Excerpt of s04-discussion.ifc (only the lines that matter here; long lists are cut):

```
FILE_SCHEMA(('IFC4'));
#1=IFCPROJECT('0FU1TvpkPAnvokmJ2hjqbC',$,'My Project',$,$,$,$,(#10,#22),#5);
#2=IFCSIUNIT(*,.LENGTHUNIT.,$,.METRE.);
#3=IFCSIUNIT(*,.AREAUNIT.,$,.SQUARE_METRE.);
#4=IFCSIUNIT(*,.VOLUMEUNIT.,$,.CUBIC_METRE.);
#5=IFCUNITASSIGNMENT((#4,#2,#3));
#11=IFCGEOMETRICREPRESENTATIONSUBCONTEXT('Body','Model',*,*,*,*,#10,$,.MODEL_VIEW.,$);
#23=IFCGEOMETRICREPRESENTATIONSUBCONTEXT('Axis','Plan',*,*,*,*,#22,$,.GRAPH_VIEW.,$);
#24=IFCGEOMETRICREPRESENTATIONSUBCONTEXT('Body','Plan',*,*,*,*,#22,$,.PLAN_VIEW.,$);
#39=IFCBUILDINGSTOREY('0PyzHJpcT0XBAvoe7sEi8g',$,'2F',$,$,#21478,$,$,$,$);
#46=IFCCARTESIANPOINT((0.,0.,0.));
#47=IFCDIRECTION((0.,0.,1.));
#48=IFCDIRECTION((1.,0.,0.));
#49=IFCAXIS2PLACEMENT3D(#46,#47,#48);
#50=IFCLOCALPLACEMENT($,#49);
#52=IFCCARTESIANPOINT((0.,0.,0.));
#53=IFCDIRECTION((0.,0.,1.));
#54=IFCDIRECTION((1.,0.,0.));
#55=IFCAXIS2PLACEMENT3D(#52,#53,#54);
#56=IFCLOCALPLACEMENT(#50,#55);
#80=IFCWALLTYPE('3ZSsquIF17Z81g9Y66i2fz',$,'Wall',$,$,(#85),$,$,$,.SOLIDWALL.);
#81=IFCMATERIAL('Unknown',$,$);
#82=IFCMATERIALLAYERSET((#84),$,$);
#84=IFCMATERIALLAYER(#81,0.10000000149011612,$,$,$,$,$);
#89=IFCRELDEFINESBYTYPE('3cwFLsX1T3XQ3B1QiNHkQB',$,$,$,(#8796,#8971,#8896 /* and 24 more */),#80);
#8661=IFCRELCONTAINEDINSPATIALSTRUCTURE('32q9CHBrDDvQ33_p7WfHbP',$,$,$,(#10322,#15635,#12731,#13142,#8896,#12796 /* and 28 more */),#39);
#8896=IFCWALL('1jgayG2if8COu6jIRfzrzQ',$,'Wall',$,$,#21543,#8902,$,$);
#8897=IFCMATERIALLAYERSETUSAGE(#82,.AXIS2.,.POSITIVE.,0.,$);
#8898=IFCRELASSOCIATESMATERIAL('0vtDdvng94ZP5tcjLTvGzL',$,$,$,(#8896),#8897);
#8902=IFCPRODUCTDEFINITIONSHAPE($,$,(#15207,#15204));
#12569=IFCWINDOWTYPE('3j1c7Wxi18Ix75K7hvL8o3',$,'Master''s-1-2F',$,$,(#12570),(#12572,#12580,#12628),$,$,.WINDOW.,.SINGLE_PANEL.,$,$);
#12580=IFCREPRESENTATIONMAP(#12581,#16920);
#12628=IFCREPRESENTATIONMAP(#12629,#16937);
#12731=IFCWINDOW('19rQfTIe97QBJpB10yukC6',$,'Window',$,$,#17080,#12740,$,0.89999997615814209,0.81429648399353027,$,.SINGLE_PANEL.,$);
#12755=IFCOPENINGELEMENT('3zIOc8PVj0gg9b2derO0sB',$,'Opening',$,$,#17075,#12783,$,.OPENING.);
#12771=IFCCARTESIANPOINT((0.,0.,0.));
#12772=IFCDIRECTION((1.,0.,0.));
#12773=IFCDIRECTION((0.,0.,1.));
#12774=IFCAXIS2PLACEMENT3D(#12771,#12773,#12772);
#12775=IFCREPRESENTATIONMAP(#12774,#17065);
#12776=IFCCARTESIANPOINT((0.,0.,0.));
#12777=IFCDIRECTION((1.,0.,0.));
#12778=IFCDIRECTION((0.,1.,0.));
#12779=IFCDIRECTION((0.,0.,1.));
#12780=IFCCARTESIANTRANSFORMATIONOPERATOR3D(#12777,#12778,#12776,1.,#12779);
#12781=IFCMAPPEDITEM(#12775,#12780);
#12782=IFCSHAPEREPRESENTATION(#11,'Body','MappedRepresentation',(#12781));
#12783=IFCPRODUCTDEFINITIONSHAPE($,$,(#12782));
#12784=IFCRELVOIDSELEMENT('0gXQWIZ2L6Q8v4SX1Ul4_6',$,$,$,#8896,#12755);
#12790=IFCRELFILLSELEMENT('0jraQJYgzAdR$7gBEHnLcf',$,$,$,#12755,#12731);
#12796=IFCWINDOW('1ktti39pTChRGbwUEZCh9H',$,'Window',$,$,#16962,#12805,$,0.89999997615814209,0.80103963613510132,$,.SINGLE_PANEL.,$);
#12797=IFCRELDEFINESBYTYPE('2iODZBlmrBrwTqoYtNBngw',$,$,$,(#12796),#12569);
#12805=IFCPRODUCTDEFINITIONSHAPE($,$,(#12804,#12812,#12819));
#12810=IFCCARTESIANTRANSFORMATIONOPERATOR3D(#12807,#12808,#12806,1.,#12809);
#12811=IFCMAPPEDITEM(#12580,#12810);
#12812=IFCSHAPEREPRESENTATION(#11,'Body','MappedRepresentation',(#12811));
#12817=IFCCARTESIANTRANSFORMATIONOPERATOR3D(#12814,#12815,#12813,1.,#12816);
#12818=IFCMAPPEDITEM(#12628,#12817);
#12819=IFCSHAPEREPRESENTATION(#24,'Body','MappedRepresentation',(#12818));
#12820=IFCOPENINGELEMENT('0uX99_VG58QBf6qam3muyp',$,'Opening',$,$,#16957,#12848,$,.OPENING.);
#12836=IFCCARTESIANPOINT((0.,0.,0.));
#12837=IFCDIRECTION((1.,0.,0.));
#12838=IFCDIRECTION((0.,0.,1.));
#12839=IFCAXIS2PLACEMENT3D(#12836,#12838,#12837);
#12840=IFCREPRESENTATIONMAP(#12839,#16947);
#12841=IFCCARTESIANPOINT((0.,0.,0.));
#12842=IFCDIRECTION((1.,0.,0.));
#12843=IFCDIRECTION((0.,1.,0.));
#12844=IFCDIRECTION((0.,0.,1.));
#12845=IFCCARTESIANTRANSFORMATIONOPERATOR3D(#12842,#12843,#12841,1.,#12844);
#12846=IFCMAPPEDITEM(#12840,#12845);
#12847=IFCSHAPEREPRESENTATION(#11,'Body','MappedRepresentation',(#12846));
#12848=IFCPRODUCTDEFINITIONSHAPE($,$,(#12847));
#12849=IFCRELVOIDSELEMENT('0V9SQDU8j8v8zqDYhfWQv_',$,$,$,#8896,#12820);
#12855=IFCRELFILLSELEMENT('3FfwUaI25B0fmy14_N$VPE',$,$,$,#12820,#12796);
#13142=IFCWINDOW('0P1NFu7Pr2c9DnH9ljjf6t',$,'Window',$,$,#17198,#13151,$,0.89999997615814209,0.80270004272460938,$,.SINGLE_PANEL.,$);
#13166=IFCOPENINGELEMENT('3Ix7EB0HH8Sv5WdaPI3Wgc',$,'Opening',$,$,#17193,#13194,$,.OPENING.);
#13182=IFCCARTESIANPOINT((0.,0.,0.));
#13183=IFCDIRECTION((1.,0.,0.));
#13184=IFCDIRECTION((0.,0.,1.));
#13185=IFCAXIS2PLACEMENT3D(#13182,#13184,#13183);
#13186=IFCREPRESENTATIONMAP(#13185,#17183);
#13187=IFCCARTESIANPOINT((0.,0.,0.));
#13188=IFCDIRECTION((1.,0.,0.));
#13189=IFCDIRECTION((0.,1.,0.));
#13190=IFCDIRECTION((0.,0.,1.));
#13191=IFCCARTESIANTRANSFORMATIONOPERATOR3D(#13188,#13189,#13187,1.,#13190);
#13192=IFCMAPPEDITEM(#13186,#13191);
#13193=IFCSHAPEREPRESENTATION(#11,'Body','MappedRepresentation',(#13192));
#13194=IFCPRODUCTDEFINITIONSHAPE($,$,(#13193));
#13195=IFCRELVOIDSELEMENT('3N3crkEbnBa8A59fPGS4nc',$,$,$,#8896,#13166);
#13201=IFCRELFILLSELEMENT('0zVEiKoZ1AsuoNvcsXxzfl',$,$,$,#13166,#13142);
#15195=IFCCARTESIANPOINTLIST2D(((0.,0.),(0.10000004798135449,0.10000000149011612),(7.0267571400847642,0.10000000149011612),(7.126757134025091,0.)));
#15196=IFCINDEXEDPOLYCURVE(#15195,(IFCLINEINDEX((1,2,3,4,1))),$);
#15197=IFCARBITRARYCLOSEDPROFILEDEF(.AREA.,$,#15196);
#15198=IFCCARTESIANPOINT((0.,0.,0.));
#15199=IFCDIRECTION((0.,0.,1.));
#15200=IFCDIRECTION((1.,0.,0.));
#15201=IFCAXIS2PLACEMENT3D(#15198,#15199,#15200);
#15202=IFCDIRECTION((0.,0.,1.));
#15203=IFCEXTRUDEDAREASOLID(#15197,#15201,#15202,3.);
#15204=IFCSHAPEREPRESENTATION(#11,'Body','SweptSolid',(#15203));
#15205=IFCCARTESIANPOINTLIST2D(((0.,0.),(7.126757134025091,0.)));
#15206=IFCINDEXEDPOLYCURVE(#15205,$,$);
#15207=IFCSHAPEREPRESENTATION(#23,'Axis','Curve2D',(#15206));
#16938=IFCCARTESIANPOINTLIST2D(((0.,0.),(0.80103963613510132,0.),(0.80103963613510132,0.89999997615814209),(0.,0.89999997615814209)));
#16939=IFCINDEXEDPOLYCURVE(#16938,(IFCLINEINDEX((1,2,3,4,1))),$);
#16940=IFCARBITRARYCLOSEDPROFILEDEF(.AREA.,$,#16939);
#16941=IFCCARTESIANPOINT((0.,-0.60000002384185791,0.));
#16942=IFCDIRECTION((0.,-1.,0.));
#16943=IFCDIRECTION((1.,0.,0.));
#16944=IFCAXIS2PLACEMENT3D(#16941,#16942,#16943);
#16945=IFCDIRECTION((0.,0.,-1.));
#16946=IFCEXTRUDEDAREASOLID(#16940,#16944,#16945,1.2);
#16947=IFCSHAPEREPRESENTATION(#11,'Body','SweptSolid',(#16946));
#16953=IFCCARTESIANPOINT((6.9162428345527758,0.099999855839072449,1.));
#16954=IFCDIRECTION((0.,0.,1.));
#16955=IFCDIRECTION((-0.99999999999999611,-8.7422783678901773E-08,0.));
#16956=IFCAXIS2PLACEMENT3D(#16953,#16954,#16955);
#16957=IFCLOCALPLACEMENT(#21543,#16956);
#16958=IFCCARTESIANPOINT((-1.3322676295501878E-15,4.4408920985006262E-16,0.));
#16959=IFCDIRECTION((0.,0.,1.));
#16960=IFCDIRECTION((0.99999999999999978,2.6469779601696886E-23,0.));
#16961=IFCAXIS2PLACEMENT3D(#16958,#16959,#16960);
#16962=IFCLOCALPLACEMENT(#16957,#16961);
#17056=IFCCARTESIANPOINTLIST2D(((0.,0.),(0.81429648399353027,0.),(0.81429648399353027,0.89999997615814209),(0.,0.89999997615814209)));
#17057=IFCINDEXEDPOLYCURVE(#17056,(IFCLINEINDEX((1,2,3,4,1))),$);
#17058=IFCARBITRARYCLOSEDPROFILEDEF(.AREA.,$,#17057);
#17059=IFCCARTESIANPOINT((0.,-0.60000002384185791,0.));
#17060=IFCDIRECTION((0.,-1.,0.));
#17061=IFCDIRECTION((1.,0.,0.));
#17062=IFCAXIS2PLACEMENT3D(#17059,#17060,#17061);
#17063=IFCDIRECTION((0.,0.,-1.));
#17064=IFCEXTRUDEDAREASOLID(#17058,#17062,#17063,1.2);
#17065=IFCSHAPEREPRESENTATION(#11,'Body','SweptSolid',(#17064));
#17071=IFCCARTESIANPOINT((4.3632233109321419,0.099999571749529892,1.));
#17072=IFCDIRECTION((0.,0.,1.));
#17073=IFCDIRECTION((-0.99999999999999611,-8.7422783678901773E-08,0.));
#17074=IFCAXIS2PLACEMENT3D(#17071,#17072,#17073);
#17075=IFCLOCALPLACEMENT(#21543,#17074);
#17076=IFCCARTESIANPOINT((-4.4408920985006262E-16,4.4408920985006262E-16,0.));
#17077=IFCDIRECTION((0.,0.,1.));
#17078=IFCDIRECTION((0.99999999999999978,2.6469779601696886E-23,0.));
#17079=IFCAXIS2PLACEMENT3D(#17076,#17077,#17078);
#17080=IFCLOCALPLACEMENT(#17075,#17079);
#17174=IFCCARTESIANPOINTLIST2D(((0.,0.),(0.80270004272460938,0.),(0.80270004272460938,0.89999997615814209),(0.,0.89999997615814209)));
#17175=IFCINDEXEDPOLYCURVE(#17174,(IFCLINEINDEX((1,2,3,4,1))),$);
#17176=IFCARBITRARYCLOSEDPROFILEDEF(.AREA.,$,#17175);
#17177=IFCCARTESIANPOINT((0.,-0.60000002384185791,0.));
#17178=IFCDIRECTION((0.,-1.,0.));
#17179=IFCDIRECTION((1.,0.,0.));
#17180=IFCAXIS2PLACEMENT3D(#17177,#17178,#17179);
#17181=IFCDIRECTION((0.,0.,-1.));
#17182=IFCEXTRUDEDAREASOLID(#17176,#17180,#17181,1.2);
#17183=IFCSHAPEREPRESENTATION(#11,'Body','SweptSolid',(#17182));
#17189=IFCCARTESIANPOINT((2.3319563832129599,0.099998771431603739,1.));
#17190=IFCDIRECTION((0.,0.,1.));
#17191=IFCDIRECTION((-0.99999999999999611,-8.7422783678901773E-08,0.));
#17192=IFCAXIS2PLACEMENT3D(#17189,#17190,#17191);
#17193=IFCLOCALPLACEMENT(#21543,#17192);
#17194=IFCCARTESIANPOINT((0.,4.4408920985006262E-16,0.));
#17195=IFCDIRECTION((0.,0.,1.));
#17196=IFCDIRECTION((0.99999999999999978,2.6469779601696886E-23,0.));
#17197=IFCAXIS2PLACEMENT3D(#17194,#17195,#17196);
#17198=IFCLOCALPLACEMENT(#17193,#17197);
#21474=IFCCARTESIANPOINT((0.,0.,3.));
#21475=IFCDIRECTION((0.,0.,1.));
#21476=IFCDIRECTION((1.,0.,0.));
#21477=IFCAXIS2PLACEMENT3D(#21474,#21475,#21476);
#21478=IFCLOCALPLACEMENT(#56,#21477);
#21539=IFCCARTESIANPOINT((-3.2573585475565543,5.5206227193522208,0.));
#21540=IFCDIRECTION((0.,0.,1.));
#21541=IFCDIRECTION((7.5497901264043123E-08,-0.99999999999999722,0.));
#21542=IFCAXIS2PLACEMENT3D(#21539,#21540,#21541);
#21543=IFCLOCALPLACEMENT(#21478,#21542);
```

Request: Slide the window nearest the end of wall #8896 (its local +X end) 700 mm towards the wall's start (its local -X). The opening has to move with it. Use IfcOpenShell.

```python
import ifcopenshell
import ifcopenshell.api.geometry
import ifcopenshell.util.placement
import ifcopenshell.util.unit

model = ifcopenshell.open("s04-discussion.ifc")
unit_scale = ifcopenshell.util.unit.calculate_unit_scale(model)

window = model.by_guid("1ktti39pTChRGbwUEZCh9H")
opening = window.FillsVoids[0].RelatingOpeningElement
wall = opening.VoidsElements[0].RelatingBuildingElement

wall_matrix = ifcopenshell.util.placement.get_local_placement(wall.ObjectPlacement)
shift = wall_matrix[:3, 0] * -0.7 / unit_scale
before = ifcopenshell.util.placement.get_local_placement(window.ObjectPlacement)[:3, 3].copy()

# The window is placed relative to its opening, so it follows when the opening moves.
matrix = ifcopenshell.util.placement.get_local_placement(opening.ObjectPlacement)
matrix[:3, 3] += shift
ifcopenshell.api.geometry.edit_object_placement(
    model, product=opening, matrix=matrix, is_si=False, should_transform_children=True
)

after = ifcopenshell.util.placement.get_local_placement(window.ObjectPlacement)[:3, 3]
print("window moved by", (after - before).round(3) + 0.0)

model.write("s04-discussion_updated.ifc")
```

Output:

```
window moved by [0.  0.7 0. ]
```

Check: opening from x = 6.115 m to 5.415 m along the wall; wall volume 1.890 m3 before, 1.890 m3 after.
